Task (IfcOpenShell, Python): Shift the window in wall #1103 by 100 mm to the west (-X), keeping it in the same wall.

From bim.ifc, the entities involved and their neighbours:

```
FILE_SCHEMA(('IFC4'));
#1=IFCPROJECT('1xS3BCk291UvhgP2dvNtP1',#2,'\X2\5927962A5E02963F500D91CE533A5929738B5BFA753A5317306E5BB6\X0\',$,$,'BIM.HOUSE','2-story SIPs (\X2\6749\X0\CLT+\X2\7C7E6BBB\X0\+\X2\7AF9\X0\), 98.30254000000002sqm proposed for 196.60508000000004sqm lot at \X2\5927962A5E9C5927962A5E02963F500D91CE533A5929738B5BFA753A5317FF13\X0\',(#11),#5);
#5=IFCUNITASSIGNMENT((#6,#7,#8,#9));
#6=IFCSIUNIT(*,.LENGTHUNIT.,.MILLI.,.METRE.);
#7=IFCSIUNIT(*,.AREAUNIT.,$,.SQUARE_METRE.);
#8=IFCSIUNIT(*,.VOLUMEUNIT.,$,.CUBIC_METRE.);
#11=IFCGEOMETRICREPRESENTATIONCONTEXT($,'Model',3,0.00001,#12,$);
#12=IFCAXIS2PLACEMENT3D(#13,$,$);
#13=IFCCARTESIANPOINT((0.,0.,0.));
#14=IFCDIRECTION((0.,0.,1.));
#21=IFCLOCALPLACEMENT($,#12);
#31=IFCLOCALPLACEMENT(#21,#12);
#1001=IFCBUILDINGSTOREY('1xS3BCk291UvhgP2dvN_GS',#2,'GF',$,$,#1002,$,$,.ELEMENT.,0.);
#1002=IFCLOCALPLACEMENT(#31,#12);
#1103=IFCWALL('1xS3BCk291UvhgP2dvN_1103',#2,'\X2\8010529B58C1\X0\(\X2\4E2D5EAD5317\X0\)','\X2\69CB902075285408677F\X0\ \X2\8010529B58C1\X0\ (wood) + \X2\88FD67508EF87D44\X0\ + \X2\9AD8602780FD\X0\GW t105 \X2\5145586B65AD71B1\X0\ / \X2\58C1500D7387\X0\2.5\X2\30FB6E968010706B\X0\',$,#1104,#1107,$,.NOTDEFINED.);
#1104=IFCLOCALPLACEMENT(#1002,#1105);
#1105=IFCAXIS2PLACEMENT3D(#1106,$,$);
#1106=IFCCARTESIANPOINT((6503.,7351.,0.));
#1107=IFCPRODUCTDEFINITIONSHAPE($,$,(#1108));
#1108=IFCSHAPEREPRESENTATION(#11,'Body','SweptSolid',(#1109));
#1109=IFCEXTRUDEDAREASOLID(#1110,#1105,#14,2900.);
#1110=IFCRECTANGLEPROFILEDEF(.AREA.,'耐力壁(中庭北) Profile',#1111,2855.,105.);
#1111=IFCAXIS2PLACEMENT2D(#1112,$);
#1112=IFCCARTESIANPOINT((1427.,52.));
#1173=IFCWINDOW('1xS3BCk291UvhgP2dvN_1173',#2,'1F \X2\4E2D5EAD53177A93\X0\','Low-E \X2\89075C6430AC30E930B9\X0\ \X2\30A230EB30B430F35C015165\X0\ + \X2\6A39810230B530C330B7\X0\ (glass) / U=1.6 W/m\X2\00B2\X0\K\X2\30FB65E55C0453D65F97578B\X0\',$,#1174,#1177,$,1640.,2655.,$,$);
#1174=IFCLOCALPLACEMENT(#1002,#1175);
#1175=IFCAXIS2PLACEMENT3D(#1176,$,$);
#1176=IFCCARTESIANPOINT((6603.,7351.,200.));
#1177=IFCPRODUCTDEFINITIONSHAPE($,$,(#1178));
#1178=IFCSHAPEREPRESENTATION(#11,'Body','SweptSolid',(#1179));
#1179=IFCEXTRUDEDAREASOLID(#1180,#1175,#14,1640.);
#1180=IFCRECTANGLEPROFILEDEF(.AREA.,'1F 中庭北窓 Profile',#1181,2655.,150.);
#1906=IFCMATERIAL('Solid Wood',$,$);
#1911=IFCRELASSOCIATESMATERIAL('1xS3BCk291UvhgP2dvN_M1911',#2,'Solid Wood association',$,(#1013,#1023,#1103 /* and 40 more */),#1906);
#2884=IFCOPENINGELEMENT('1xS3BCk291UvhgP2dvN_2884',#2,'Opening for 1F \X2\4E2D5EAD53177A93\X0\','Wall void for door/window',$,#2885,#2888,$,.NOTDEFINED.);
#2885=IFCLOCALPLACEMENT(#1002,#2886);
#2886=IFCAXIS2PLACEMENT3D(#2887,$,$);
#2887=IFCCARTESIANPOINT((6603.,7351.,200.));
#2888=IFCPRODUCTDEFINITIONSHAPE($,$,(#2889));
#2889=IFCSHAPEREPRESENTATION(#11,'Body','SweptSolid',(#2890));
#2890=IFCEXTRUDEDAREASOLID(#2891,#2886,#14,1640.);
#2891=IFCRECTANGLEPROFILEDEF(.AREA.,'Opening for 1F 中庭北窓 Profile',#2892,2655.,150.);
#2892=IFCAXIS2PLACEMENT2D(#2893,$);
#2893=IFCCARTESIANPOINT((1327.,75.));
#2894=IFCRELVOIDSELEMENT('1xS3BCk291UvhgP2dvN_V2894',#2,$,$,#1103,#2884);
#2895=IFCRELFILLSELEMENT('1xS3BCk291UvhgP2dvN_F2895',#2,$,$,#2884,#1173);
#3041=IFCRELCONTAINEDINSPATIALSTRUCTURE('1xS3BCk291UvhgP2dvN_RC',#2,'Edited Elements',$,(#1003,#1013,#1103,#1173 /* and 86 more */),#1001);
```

```python
import ifcopenshell
import ifcopenshell.api.geometry
import ifcopenshell.util.placement

model = ifcopenshell.open("bim.ifc")

window = model.by_id(1173)
opening = window.FillsVoids[0].RelatingOpeningElement
wall = opening.VoidsElements[0].RelatingBuildingElement

wall_matrix = ifcopenshell.util.placement.get_local_placement(wall.ObjectPlacement)
shift = wall_matrix[:3, 0] * -100.0
before = ifcopenshell.util.placement.get_local_placement(window.ObjectPlacement)[:3, 3].copy()

# The window is not placed relative to its opening, so move both.
for product in (opening, window):
    matrix = ifcopenshell.util.placement.get_local_placement(product.ObjectPlacement)
    matrix[:3, 3] += shift
    ifcopenshell.api.geometry.edit_object_placement(model, product=product, matrix=matrix, is_si=False)

after = ifcopenshell.util.placement.get_local_placement(window.ObjectPlacement)[:3, 3]
print("window moved by", (after - before).round(3) + 0.0)

model.write("bim_rev.ifc")
```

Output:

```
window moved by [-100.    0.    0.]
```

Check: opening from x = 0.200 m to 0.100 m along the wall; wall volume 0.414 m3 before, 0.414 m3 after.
